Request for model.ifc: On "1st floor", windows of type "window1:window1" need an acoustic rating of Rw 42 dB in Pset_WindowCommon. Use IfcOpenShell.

First a look at what the model holds.

```python
import ifcopenshell
import ifcopenshell.util.element

model = ifcopenshell.open("model.ifc")
print(model.schema)
storey = next(s for s in model.by_type("IfcBuildingStorey") if s.Name == "1st floor")
windows = [e for e in ifcopenshell.util.element.get_decomposition(storey) if e.is_a("IfcWindow")]
seen = {}
for e in windows:
    element_type = ifcopenshell.util.element.get_type(e)
    key = (element_type.Name if element_type != e and element_type else None, ifcopenshell.util.element.get_pset(e, "Pset_WindowCommon", "AcousticRating"))
    seen[key] = seen.get(key, 0) + 1
for (name, value), count in sorted(seen.items(), key=str):
    print(count, "x", name, "|", value)
```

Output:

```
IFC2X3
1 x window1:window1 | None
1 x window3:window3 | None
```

```python
import ifcopenshell
import ifcopenshell.api.pset
import ifcopenshell.util.element

model = ifcopenshell.open("model.ifc")

storey = next(s for s in model.by_type("IfcBuildingStorey") if s.Name == "1st floor")
windows = [e for e in ifcopenshell.util.element.get_decomposition(storey) if e.is_a("IfcWindow")]

count = 0
for e in windows:
    element_type = ifcopenshell.util.element.get_type(e)
    if element_type in (None, e) or element_type.Name != "window1:window1":
        continue
    # add_pset returns the element's existing set when there is one.
    pset = ifcopenshell.api.pset.add_pset(model, product=e, name="Pset_WindowCommon")
    ifcopenshell.api.pset.edit_pset(model, pset=pset, properties={"AcousticRating": "Rw 42 dB"})
    count += 1

print(count, "windows updated")

model.write("model-out.ifc")
```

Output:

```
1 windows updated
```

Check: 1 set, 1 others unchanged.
